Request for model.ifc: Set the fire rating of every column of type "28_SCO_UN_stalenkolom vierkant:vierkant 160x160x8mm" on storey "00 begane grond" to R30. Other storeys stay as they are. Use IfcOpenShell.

First a look at what the model holds.

```python
import ifcopenshell
import ifcopenshell.util.element

model = ifcopenshell.open("model.ifc")
print(model.schema)
storey = next(s for s in model.by_type("IfcBuildingStorey") if s.Name == "00 begane grond")
columns = [e for e in ifcopenshell.util.element.get_decomposition(storey) if e.is_a("IfcColumn")]
seen = {}
for e in columns:
    element_type = ifcopenshell.util.element.get_type(e)
    key = (element_type.Name if element_type != e and element_type else None, ifcopenshell.util.element.get_pset(e, "Pset_ColumnCommon", "FireRating"))
    seen[key] = seen.get(key, 0) + 1
for (name, value), count in sorted(seen.items(), key=str):
    print(count, "x", name, "|", value)
```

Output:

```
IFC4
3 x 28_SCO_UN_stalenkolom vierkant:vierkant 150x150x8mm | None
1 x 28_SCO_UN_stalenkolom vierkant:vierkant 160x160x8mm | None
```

```python
import ifcopenshell
import ifcopenshell.api.pset
import ifcopenshell.util.element

model = ifcopenshell.open("model.ifc")

storey = next(s for s in model.by_type("IfcBuildingStorey") if s.Name == "00 begane grond")
columns = [e for e in ifcopenshell.util.element.get_decomposition(storey) if e.is_a("IfcColumn")]

count = 0
for e in columns:
    element_type = ifcopenshell.util.element.get_type(e)
    if element_type in (None, e) or element_type.Name != "28_SCO_UN_stalenkolom vierkant:vierkant 160x160x8mm":
        continue
    # add_pset returns the element's existing set when there is one.
    pset = ifcopenshell.api.pset.add_pset(model, product=e, name="Pset_ColumnCommon")
    ifcopenshell.api.pset.edit_pset(model, pset=pset, properties={"FireRating": "R30"})
    count += 1

print(count, "columns updated")

model.write("model_v2.ifc")
```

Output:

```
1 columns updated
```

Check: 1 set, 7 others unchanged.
